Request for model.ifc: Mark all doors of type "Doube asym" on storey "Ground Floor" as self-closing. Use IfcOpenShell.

First a look at what the model holds.

```python
import ifcopenshell
import ifcopenshell.util.element

model = ifcopenshell.open("model.ifc")
print(model.schema)
storey = next(s for s in model.by_type("IfcBuildingStorey") if s.Name == "Ground Floor")
doors = [e for e in ifcopenshell.util.element.get_decomposition(storey) if e.is_a("IfcDoor")]
seen = {}
for e in doors:
    element_type = ifcopenshell.util.element.get_type(e)
    key = (element_type.Name if element_type != e and element_type else None, ifcopenshell.util.element.get_pset(e, "Pset_DoorCommon", "SelfClosing"))
    seen[key] = seen.get(key, 0) + 1
for (name, value), count in sorted(seen.items(), key=str):
    print(count, "x", name, "|", value)
```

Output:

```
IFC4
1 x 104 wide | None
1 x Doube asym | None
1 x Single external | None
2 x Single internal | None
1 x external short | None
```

```python
import ifcopenshell
import ifcopenshell.api.pset
import ifcopenshell.util.element

model = ifcopenshell.open("model.ifc")

storey = next(s for s in model.by_type("IfcBuildingStorey") if s.Name == "Ground Floor")
doors = [e for e in ifcopenshell.util.element.get_decomposition(storey) if e.is_a("IfcDoor")]

count = 0
for e in doors:
    element_type = ifcopenshell.util.element.get_type(e)
    if element_type in (None, e) or element_type.Name != "Doube asym":
        continue
    # add_pset returns the element's existing set when there is one.
    pset = ifcopenshell.api.pset.add_pset(model, product=e, name="Pset_DoorCommon")
    ifcopenshell.api.pset.edit_pset(model, pset=pset, properties={"SelfClosing": True})
    count += 1

print(count, "doors updated")

model.write("model_v2.ifc")
```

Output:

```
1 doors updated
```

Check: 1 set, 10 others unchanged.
